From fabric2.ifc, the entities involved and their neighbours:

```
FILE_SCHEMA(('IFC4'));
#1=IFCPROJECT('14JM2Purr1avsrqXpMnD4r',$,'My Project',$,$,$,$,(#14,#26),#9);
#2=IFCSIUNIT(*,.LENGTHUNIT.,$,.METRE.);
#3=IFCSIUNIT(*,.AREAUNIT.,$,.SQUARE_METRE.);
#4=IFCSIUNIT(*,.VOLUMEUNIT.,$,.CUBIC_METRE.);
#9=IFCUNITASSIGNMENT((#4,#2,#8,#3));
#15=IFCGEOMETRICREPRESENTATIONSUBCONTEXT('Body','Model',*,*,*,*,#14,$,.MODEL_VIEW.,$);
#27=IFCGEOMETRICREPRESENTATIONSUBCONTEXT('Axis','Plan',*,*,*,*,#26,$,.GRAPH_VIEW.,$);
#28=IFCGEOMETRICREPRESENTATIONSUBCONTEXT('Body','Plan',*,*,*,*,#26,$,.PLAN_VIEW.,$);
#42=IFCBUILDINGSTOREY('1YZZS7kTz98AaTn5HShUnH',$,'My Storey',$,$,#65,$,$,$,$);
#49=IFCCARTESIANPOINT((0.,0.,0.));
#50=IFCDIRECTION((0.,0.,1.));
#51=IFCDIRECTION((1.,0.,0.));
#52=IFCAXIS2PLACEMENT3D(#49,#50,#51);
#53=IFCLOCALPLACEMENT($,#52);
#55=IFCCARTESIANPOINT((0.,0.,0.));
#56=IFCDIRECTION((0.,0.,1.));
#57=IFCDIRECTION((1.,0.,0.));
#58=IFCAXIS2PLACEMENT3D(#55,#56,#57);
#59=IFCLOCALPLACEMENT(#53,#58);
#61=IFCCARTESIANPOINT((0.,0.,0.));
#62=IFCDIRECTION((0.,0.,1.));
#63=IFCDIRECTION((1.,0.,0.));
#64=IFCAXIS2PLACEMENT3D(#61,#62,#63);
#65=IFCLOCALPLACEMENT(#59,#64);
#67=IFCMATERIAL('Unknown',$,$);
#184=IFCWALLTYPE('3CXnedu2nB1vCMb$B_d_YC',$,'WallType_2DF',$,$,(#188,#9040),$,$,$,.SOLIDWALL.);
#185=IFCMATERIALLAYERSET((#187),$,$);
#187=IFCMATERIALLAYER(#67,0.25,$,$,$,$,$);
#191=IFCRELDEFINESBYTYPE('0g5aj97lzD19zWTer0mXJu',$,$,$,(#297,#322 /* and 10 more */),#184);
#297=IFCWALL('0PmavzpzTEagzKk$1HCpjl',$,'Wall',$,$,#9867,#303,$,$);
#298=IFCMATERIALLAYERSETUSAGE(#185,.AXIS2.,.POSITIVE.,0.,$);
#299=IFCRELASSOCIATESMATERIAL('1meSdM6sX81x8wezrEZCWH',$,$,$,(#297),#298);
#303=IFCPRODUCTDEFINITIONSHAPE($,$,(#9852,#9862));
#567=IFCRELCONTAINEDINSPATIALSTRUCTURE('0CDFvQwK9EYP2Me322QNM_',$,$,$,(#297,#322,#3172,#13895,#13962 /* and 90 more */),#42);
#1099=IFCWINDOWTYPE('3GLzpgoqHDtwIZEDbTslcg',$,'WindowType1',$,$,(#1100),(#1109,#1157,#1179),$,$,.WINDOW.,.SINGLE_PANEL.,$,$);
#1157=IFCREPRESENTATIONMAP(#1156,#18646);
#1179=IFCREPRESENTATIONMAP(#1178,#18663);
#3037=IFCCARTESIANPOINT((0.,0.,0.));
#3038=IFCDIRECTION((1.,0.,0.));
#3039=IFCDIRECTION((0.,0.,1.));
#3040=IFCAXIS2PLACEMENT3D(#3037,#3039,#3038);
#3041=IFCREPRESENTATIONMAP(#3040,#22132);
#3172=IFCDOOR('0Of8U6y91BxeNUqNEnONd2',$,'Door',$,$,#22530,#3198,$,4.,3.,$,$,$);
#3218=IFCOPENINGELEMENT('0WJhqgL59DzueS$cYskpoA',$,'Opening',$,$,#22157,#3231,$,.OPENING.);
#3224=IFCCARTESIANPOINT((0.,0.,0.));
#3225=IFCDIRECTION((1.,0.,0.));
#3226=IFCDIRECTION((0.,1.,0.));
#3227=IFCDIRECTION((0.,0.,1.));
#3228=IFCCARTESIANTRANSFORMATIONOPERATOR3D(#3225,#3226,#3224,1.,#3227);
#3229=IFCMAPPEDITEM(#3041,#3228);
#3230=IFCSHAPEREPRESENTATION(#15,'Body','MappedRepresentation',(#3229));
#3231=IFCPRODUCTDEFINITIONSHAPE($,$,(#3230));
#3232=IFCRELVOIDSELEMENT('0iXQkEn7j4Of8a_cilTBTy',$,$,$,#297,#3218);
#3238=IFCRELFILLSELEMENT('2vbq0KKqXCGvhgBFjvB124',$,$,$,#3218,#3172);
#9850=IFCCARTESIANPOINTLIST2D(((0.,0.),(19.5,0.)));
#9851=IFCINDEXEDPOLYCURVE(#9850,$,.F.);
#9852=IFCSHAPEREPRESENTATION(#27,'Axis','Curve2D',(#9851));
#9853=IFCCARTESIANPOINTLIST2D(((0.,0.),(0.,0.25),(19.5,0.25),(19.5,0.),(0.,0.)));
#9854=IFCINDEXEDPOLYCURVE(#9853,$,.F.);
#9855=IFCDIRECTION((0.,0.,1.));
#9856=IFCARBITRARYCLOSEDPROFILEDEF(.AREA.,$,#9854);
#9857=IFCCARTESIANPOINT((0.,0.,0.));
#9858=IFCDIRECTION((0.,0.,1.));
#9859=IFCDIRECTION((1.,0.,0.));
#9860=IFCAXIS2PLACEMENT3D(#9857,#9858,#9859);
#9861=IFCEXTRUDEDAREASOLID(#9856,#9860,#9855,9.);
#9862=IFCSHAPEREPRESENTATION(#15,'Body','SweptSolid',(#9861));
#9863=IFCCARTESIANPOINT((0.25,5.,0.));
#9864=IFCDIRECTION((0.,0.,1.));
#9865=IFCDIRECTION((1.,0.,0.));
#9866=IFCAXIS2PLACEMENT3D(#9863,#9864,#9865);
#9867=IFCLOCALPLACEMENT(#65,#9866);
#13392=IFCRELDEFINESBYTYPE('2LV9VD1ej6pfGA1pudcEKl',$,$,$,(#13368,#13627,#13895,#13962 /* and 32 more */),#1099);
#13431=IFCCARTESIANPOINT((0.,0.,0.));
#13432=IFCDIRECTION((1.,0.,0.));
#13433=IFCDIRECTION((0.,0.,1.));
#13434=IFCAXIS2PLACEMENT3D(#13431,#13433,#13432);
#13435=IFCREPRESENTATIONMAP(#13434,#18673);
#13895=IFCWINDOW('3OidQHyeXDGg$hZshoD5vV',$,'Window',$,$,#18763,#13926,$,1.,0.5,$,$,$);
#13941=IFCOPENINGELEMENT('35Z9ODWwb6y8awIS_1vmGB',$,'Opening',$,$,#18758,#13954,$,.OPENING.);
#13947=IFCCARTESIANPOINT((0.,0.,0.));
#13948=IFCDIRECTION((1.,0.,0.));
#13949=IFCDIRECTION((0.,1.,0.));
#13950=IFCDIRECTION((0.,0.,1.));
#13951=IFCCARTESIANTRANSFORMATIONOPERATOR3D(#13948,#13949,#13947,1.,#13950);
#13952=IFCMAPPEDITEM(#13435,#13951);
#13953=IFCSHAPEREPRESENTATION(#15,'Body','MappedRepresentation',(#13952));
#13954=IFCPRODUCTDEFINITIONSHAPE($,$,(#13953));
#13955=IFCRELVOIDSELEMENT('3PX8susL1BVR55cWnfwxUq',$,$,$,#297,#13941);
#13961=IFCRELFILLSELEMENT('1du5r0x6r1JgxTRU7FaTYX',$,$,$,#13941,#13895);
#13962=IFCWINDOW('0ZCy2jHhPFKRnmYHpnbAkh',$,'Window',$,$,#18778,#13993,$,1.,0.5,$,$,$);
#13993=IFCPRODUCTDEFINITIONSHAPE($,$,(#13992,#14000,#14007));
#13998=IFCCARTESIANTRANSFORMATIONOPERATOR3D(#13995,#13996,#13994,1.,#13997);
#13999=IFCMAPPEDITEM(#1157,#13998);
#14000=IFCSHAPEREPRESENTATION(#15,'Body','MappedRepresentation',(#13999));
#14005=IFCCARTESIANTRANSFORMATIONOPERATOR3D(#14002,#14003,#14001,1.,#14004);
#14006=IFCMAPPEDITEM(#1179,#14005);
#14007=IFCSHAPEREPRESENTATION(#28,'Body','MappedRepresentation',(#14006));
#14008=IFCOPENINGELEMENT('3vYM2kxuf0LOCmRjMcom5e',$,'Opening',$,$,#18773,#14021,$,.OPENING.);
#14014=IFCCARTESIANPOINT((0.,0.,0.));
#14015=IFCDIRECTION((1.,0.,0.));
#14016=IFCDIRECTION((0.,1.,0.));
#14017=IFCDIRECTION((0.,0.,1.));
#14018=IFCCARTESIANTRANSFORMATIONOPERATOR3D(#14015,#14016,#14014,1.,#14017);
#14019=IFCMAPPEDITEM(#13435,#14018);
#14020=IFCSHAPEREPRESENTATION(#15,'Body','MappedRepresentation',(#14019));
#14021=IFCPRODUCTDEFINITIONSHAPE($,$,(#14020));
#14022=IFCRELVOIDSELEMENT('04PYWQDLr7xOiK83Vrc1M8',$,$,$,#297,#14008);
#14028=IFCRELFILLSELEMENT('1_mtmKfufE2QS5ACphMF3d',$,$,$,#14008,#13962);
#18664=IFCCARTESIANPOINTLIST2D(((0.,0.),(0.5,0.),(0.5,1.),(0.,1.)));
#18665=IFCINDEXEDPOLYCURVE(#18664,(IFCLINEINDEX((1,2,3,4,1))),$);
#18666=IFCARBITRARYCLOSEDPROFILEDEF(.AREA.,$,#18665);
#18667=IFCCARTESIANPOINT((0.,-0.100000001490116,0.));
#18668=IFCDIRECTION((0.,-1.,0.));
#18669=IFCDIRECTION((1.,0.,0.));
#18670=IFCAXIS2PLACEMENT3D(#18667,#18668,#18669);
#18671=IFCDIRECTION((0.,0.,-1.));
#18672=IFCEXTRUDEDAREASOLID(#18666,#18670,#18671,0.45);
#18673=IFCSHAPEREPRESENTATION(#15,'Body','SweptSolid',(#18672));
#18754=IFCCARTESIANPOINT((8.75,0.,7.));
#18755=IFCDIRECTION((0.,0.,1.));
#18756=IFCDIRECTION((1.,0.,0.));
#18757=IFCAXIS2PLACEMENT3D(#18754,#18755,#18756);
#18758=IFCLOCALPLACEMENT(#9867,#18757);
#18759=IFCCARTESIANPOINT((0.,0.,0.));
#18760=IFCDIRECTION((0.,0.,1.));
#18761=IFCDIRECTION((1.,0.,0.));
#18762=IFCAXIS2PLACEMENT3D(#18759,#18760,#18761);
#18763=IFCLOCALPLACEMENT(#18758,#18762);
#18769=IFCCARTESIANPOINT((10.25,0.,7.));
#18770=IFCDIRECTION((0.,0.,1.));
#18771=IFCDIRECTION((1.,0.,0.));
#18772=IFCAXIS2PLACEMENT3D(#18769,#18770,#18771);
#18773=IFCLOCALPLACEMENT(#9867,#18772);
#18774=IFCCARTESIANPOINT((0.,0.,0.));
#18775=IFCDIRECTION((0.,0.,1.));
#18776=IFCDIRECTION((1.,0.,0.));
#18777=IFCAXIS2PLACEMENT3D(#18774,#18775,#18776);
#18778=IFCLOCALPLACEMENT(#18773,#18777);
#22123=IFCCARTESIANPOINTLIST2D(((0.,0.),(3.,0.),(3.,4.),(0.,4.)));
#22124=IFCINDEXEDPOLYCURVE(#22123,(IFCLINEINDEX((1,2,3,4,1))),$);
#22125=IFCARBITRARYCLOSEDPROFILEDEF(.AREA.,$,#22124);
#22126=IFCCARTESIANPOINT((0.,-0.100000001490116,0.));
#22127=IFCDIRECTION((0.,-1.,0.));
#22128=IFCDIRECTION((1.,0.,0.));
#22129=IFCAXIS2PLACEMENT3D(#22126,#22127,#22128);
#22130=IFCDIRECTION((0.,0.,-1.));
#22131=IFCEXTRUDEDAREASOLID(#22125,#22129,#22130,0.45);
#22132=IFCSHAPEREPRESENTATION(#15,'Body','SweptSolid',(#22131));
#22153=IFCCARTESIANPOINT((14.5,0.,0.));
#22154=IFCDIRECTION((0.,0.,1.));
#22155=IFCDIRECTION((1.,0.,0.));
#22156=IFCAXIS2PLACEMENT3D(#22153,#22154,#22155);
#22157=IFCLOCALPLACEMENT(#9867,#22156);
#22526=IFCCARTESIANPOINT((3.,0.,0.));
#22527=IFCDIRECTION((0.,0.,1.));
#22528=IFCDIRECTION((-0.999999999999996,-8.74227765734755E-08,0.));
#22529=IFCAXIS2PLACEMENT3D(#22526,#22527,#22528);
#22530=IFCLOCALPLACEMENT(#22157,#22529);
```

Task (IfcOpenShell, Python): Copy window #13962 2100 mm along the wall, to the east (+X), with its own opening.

```python
import ifcopenshell
import ifcopenshell.api.feature
import ifcopenshell.api.geometry
import ifcopenshell.api.root
import ifcopenshell.geom
import ifcopenshell.util.element
import ifcopenshell.util.placement
import ifcopenshell.util.shape
import ifcopenshell.util.unit

model = ifcopenshell.open("fabric2.ifc")
unit_scale = ifcopenshell.util.unit.calculate_unit_scale(model)
settings = ifcopenshell.geom.settings()


def volume(element):
    """Net volume in cubic metres, openings subtracted."""
    shape = ifcopenshell.geom.create_shape(settings, element)
    return ifcopenshell.util.shape.get_volume(shape.geometry)


window = model.by_guid("0ZCy2jHhPFKRnmYHpnbAkh")
opening = window.FillsVoids[0].RelatingOpeningElement
wall = opening.VoidsElements[0].RelatingBuildingElement
before = volume(wall)
shift = ifcopenshell.util.placement.get_local_placement(wall.ObjectPlacement)[:3, 0] * 2.1 / unit_scale

# copy_class copies the void relationship, type, container and properties, but no geometry.
new_opening = ifcopenshell.api.root.copy_class(model, product=opening)
new_opening.Representation = ifcopenshell.util.element.copy_deep(
    model, opening.Representation, exclude=["IfcGeometricRepresentationContext", "IfcRepresentationMap"]
)
new_window = ifcopenshell.api.root.copy_class(model, product=window)
new_window.Representation = ifcopenshell.util.element.copy_deep(
    model, window.Representation, exclude=["IfcGeometricRepresentationContext", "IfcRepresentationMap"]
)
ifcopenshell.api.feature.add_filling(model, opening=new_opening, element=new_window)

for old, new in ((opening, new_opening), (window, new_window)):
    matrix = ifcopenshell.util.placement.get_local_placement(old.ObjectPlacement)
    matrix[:3, 3] += shift
    ifcopenshell.api.geometry.edit_object_placement(model, product=new, matrix=matrix, is_si=False)

after = volume(wall)

print(f"wall volume {before:.3f} -> {after:.3f} m3")

model.write("fabric2-out.ifc")
```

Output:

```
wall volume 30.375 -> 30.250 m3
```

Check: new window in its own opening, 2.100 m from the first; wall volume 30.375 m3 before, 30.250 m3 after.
